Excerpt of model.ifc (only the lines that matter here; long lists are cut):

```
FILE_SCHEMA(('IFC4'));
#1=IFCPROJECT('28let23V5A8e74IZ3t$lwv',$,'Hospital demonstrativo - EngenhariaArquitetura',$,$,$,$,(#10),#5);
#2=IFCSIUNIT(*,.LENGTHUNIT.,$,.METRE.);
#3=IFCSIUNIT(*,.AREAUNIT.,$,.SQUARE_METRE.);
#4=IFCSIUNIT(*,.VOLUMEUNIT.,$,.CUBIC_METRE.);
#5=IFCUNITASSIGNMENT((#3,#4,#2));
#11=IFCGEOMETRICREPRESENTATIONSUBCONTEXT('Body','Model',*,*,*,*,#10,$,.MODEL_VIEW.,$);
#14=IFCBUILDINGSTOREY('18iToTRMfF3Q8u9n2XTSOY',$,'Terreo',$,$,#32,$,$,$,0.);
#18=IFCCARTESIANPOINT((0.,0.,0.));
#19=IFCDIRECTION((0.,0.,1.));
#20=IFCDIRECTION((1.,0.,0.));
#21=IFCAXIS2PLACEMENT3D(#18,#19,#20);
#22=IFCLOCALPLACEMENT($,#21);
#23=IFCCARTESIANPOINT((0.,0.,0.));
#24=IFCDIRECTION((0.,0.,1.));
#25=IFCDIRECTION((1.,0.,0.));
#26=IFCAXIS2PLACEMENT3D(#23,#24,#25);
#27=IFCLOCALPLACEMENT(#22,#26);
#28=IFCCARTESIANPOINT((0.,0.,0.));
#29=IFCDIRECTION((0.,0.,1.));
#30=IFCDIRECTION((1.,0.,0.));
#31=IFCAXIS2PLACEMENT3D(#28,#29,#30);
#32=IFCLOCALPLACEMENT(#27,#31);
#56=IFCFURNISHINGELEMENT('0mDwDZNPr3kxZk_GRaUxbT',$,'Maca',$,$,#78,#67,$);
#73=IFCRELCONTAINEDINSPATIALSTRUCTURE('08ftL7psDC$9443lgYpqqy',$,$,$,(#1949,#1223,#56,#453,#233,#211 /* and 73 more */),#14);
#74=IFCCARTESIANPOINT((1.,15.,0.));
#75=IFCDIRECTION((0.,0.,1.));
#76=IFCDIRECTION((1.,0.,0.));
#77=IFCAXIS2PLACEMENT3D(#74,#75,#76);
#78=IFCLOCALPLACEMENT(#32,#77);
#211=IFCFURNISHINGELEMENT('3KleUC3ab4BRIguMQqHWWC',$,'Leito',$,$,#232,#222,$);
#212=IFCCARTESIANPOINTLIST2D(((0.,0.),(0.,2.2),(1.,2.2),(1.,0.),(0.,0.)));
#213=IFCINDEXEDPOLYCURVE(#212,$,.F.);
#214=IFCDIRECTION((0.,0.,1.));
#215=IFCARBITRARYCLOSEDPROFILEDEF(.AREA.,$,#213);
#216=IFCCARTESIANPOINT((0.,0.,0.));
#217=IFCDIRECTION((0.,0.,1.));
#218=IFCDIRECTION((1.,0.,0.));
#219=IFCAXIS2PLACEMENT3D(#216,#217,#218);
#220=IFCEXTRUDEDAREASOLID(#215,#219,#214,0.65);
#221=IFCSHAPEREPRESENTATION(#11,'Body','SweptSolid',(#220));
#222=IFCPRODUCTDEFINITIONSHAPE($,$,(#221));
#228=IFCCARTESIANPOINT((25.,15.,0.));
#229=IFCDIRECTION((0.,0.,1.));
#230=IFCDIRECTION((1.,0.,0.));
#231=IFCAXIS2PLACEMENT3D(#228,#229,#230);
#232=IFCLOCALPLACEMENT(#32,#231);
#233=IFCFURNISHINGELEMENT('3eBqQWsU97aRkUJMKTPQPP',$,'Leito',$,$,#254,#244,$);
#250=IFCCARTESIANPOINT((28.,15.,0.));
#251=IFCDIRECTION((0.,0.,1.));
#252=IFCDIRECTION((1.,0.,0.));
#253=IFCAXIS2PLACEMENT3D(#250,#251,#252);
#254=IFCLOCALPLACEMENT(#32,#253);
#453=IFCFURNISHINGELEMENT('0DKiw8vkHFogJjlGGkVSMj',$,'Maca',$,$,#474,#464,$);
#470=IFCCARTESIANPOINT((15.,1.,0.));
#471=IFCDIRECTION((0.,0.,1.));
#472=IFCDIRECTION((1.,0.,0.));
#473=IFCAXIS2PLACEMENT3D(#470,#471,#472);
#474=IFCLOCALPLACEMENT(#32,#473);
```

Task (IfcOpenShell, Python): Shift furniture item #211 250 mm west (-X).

```python
import ifcopenshell
import ifcopenshell.api.geometry
import ifcopenshell.util.placement

model = ifcopenshell.open("model.ifc")

item = model.by_id(211)
matrix = ifcopenshell.util.placement.get_local_placement(item.ObjectPlacement)
matrix[0, 3] -= 0.25
ifcopenshell.api.geometry.edit_object_placement(model, product=item, matrix=matrix, is_si=False)

print(ifcopenshell.util.placement.get_local_placement(item.ObjectPlacement).round(3) + 0.0)

model.write("model_rev.ifc")
```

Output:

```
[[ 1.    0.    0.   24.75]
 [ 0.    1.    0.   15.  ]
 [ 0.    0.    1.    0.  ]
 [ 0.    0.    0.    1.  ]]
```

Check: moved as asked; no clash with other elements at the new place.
